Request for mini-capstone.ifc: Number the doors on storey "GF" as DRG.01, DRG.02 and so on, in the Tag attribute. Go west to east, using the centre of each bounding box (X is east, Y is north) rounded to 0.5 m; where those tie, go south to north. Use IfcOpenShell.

First a look at what the model holds.

```python
import ifcopenshell
import ifcopenshell.util.element
import ifcopenshell.util.placement

model = ifcopenshell.open("mini-capstone.ifc")
print(model.schema)
storey = next(s for s in model.by_type("IfcBuildingStorey") if s.Name == "GF")
doors = [e for e in ifcopenshell.util.element.get_decomposition(storey) if e.is_a("IfcDoor")]
for e in sorted(doors, key=lambda e: e.id()):
    origin = ifcopenshell.util.placement.get_local_placement(e.ObjectPlacement)[:3, 3]
    print(e.id(), e.Tag, e.Name, origin.round(2) + 0.0, sep=" | ")
```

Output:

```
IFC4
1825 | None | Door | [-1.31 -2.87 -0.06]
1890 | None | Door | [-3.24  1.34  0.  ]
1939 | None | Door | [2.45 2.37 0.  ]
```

```python
import ifcopenshell
import ifcopenshell.geom
import ifcopenshell.util.element
import ifcopenshell.util.shape

model = ifcopenshell.open("mini-capstone.ifc")
settings = ifcopenshell.geom.settings()
settings.set("use-world-coords", True)


def centre(element):
    shape = ifcopenshell.geom.create_shape(settings, element)
    return ifcopenshell.util.shape.get_bbox_centroid(shape.geometry)


storey = next(s for s in model.by_type("IfcBuildingStorey") if s.Name == "GF")
doors = [e for e in ifcopenshell.util.element.get_decomposition(storey) if e.is_a("IfcDoor")]

# Insertion points can sit at a corner or the storey origin, so sort by the geometry (in metres).
centres = {e: centre(e) for e in doors}
doors.sort(key=lambda e: (round(centres[e][0] / 0.5), centres[e][1]))

for i, e in enumerate(doors, start=1):
    number = f"DRG.{i:02d}"
    e.Tag = number
    print(e.id(), number)

model.write("mini-capstone_edited.ifc")
```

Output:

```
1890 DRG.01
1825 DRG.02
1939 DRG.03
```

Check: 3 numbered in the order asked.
